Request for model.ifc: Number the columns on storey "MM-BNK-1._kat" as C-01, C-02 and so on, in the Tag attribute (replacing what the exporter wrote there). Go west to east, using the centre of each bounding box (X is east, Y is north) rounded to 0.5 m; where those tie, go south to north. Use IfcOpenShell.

First a look at what the model holds.

```python
import ifcopenshell
import ifcopenshell.util.element
import ifcopenshell.util.placement

model = ifcopenshell.open("model.ifc")
print(model.schema)
storey = next(s for s in model.by_type("IfcBuildingStorey") if s.Name == "MM-BNK-1._kat")
columns = [e for e in ifcopenshell.util.element.get_decomposition(storey) if e.is_a("IfcColumn")]
for e in sorted(columns, key=lambda e: e.id()):
    origin = ifcopenshell.util.placement.get_local_placement(e.ObjectPlacement)[:3, 3]
    print(e.id(), e.Tag, e.Name, origin.round(2) + 0.0, sep=" | ")
```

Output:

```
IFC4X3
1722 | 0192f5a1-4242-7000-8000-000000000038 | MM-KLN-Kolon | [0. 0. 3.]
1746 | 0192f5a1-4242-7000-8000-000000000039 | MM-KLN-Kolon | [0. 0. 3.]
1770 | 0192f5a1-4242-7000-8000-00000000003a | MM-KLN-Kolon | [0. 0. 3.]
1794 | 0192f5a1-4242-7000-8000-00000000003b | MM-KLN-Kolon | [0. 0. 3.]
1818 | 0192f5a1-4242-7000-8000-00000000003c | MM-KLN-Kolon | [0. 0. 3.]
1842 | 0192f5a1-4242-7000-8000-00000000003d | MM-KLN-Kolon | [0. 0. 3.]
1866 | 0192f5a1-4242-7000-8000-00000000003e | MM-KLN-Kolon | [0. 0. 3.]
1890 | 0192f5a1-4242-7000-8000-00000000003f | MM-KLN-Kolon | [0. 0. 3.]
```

```python
import ifcopenshell
import ifcopenshell.geom
import ifcopenshell.util.element
import ifcopenshell.util.shape

model = ifcopenshell.open("model.ifc")
settings = ifcopenshell.geom.settings()
settings.set("use-world-coords", True)


def centre(element):
    shape = ifcopenshell.geom.create_shape(settings, element)
    return ifcopenshell.util.shape.get_bbox_centroid(shape.geometry)


storey = next(s for s in model.by_type("IfcBuildingStorey") if s.Name == "MM-BNK-1._kat")
columns = [e for e in ifcopenshell.util.element.get_decomposition(storey) if e.is_a("IfcColumn")]

# Insertion points can sit at a corner or the storey origin, so sort by the geometry (in metres).
centres = {e: centre(e) for e in columns}
columns.sort(key=lambda e: (round(centres[e][0] / 0.5), centres[e][1]))

for i, e in enumerate(columns, start=1):
    number = f"C-{i:02d}"
    e.Tag = number
    print(e.id(), number)

model.write("model_updated.ifc")
```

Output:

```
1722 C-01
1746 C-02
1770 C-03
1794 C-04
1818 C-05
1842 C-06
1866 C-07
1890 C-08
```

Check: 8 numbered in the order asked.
